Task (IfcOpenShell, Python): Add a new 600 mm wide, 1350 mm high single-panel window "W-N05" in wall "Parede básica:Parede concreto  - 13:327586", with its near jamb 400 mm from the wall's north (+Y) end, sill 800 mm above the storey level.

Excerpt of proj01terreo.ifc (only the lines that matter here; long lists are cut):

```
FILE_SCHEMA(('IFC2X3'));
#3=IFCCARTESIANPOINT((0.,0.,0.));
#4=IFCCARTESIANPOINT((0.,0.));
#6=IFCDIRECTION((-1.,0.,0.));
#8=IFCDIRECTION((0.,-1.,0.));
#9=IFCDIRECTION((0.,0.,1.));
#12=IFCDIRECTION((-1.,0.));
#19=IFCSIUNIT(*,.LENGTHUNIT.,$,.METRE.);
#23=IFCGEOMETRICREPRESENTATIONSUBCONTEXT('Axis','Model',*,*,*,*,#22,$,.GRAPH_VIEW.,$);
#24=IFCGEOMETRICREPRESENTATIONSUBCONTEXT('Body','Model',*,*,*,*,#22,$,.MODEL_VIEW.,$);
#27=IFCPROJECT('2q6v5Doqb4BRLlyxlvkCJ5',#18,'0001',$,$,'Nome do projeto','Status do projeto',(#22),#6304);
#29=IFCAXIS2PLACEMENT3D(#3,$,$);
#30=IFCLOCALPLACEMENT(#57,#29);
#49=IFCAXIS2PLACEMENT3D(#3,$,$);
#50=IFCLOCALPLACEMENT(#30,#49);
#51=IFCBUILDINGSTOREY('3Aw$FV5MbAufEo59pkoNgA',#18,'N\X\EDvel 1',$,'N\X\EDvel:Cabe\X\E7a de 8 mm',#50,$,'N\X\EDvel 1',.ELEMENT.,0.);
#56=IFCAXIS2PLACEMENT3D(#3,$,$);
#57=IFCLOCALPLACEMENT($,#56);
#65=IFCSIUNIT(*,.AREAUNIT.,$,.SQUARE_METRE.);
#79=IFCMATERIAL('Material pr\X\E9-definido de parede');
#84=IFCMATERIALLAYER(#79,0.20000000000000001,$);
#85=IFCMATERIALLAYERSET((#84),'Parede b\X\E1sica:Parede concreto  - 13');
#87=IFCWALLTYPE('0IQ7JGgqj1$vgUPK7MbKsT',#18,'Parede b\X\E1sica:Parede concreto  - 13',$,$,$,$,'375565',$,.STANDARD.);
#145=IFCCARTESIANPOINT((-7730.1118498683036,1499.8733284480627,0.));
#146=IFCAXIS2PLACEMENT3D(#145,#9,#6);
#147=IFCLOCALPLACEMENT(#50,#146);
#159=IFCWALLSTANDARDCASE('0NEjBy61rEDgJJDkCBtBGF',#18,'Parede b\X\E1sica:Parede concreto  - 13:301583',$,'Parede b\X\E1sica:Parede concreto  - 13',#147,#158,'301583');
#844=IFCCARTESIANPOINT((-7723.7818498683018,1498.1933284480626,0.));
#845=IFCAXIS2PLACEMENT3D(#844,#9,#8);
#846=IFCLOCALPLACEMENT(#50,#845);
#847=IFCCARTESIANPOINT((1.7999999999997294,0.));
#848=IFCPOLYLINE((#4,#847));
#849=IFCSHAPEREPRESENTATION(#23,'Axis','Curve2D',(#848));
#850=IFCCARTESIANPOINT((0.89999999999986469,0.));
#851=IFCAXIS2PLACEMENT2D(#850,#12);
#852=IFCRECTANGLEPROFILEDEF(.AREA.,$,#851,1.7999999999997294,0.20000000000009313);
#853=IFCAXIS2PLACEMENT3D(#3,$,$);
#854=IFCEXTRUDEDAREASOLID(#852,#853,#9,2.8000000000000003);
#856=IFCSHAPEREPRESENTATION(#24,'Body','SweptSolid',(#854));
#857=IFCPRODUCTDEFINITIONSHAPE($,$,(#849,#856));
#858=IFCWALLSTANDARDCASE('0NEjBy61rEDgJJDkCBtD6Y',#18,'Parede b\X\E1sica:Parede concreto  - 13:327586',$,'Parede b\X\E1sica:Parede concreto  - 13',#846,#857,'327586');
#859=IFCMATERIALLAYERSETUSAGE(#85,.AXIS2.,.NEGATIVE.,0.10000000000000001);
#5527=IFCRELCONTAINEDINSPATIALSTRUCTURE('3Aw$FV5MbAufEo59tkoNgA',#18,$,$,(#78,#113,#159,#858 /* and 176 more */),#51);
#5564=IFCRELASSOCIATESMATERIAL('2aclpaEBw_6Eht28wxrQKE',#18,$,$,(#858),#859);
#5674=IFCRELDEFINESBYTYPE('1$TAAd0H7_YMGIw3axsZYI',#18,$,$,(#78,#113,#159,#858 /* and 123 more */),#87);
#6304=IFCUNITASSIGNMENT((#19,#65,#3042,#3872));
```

```python
import numpy as np
import ifcopenshell
import ifcopenshell.api.feature
import ifcopenshell.api.geometry
import ifcopenshell.api.root
import ifcopenshell.api.spatial
import ifcopenshell.api.type
import ifcopenshell.geom
import ifcopenshell.util.element
import ifcopenshell.util.placement
import ifcopenshell.util.representation
import ifcopenshell.util.shape
import ifcopenshell.util.unit

model = ifcopenshell.open("proj01terreo.ifc")
unit_scale = ifcopenshell.util.unit.calculate_unit_scale(model)
settings = ifcopenshell.geom.settings()


def volume(element):
    """Net volume in cubic metres, openings subtracted."""
    shape = ifcopenshell.geom.create_shape(settings, element)
    return ifcopenshell.util.shape.get_volume(shape.geometry)


wall = model.by_id(858)
storey = ifcopenshell.util.element.get_container(wall, ifc_class="IfcBuildingStorey")
context = ifcopenshell.util.representation.get_context(model, "Model", "Body", "MODEL_VIEW")
before = volume(wall)

width, height, from_end, sill = 0.6, 1.35, 0.4, 0.8  # metres

# The wall runs along its own X axis, and the end named is its -X end.
wall_shape = ifcopenshell.geom.create_shape(settings, wall)
x, y, z = ifcopenshell.util.shape.get_vertices(wall_shape.geometry).T
start = x.min() + from_end
face, thickness = float(y.min()), float(y.max() - y.min())
wall_matrix = ifcopenshell.util.placement.get_local_placement(wall.ObjectPlacement)
level = ifcopenshell.util.placement.get_local_placement(storey.ObjectPlacement)[2, 3]


def in_wall(x, y):
    """Placement at x, y metres in the wall's axes, at sill height."""
    matrix = wall_matrix.copy()
    matrix[:, 3] = wall_matrix @ np.array([x / unit_scale, y / unit_scale, 0.0, 1.0])
    matrix[2, 3] = level + sill / unit_scale
    return matrix


# Opening: a box that overshoots both wall faces by 50 mm.
opening = ifcopenshell.api.root.create_entity(model, ifc_class="IfcOpeningElement")
box = ifcopenshell.api.geometry.add_wall_representation(
    model, context=context, length=width, height=height, thickness=thickness + 0.1
)
ifcopenshell.api.geometry.assign_representation(model, product=opening, representation=box)
ifcopenshell.api.geometry.edit_object_placement(model, product=opening, matrix=in_wall(start, face - 0.05), is_si=False)
ifcopenshell.api.feature.add_feature(model, feature=opening, element=wall)

window = ifcopenshell.api.root.create_entity(model, ifc_class="IfcWindow", name="W-N05")
window.OverallWidth, window.OverallHeight = width / unit_scale, height / unit_scale
body = ifcopenshell.api.geometry.add_window_representation(
    model,
    context=context,
    overall_width=window.OverallWidth,
    overall_height=window.OverallHeight,
    partition_type="SINGLE_PANEL",
)
ifcopenshell.api.geometry.assign_representation(model, product=window, representation=body)
ifcopenshell.api.spatial.assign_container(model, products=[window], relating_structure=storey)
fills = ifcopenshell.api.feature.add_filling(model, opening=opening, element=window)
fills.OwnerHistory = window.OwnerHistory  # required in IFC2X3

# IFC2X3 keeps the operation on the window style.
style = ifcopenshell.api.root.create_entity(model, ifc_class="IfcWindowStyle", name="W-N05")
style.OperationType, style.ConstructionType = "SINGLE_PANEL", "NOTDEFINED"
style.ParameterTakesPrecedence = style.Sizeable = False
ifcopenshell.api.type.assign_type(model, related_objects=[window], relating_type=style)

# Centre the window in the wall's thickness.
ifcopenshell.api.geometry.edit_object_placement(model, product=window, matrix=in_wall(start, face), is_si=False)
window_shape = ifcopenshell.geom.create_shape(settings, window)
depth = ifcopenshell.util.shape.get_vertices(window_shape.geometry)[:, 1]
offset = face + thickness / 2 - (depth.min() + depth.max()) / 2
ifcopenshell.api.geometry.edit_object_placement(model, product=window, matrix=in_wall(start, offset), is_si=False)

after = volume(wall)

print(f"wall volume {before:.3f} -> {after:.3f} m3")

model.write("proj01terreo_updated.ifc")
```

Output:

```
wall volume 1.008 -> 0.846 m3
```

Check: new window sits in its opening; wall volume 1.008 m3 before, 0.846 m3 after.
